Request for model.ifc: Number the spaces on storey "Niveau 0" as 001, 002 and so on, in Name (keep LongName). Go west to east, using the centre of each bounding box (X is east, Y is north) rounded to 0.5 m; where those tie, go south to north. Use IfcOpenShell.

First a look at what the model holds.

```python
import ifcopenshell
import ifcopenshell.util.element
import ifcopenshell.util.placement

model = ifcopenshell.open("model.ifc")
print(model.schema)
storey = next(s for s in model.by_type("IfcBuildingStorey") if s.Name == "Niveau 0")
spaces = [e for e in ifcopenshell.util.element.get_decomposition(storey) if e.is_a("IfcSpace")]
for e in sorted(spaces, key=lambda e: e.id()):
    origin = ifcopenshell.util.placement.get_local_placement(e.ObjectPlacement)[:3, 3]
    print(e.id(), e.Name, e.LongName, origin.round(2) + 0.0, sep=" | ")
```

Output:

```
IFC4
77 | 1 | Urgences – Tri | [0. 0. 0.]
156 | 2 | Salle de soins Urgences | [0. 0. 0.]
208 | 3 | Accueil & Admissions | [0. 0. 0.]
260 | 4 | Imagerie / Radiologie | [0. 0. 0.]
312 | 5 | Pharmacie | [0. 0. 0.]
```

```python
import ifcopenshell
import ifcopenshell.geom
import ifcopenshell.util.element
import ifcopenshell.util.shape

model = ifcopenshell.open("model.ifc")
settings = ifcopenshell.geom.settings()
settings.set("use-world-coords", True)


def centre(element):
    shape = ifcopenshell.geom.create_shape(settings, element)
    return ifcopenshell.util.shape.get_bbox_centroid(shape.geometry)


storey = next(s for s in model.by_type("IfcBuildingStorey") if s.Name == "Niveau 0")
spaces = [e for e in ifcopenshell.util.element.get_decomposition(storey) if e.is_a("IfcSpace")]

# Insertion points can sit at a corner or the storey origin, so sort by the geometry (in metres).
centres = {e: centre(e) for e in spaces}
spaces.sort(key=lambda e: (round(centres[e][0] / 0.5), centres[e][1]))

for i, e in enumerate(spaces, start=1):
    number = f"0{i:02d}"
    e.Name = number
    print(e.id(), number)

model.write("model_rev.ifc")
```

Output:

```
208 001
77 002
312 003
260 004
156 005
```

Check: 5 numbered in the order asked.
